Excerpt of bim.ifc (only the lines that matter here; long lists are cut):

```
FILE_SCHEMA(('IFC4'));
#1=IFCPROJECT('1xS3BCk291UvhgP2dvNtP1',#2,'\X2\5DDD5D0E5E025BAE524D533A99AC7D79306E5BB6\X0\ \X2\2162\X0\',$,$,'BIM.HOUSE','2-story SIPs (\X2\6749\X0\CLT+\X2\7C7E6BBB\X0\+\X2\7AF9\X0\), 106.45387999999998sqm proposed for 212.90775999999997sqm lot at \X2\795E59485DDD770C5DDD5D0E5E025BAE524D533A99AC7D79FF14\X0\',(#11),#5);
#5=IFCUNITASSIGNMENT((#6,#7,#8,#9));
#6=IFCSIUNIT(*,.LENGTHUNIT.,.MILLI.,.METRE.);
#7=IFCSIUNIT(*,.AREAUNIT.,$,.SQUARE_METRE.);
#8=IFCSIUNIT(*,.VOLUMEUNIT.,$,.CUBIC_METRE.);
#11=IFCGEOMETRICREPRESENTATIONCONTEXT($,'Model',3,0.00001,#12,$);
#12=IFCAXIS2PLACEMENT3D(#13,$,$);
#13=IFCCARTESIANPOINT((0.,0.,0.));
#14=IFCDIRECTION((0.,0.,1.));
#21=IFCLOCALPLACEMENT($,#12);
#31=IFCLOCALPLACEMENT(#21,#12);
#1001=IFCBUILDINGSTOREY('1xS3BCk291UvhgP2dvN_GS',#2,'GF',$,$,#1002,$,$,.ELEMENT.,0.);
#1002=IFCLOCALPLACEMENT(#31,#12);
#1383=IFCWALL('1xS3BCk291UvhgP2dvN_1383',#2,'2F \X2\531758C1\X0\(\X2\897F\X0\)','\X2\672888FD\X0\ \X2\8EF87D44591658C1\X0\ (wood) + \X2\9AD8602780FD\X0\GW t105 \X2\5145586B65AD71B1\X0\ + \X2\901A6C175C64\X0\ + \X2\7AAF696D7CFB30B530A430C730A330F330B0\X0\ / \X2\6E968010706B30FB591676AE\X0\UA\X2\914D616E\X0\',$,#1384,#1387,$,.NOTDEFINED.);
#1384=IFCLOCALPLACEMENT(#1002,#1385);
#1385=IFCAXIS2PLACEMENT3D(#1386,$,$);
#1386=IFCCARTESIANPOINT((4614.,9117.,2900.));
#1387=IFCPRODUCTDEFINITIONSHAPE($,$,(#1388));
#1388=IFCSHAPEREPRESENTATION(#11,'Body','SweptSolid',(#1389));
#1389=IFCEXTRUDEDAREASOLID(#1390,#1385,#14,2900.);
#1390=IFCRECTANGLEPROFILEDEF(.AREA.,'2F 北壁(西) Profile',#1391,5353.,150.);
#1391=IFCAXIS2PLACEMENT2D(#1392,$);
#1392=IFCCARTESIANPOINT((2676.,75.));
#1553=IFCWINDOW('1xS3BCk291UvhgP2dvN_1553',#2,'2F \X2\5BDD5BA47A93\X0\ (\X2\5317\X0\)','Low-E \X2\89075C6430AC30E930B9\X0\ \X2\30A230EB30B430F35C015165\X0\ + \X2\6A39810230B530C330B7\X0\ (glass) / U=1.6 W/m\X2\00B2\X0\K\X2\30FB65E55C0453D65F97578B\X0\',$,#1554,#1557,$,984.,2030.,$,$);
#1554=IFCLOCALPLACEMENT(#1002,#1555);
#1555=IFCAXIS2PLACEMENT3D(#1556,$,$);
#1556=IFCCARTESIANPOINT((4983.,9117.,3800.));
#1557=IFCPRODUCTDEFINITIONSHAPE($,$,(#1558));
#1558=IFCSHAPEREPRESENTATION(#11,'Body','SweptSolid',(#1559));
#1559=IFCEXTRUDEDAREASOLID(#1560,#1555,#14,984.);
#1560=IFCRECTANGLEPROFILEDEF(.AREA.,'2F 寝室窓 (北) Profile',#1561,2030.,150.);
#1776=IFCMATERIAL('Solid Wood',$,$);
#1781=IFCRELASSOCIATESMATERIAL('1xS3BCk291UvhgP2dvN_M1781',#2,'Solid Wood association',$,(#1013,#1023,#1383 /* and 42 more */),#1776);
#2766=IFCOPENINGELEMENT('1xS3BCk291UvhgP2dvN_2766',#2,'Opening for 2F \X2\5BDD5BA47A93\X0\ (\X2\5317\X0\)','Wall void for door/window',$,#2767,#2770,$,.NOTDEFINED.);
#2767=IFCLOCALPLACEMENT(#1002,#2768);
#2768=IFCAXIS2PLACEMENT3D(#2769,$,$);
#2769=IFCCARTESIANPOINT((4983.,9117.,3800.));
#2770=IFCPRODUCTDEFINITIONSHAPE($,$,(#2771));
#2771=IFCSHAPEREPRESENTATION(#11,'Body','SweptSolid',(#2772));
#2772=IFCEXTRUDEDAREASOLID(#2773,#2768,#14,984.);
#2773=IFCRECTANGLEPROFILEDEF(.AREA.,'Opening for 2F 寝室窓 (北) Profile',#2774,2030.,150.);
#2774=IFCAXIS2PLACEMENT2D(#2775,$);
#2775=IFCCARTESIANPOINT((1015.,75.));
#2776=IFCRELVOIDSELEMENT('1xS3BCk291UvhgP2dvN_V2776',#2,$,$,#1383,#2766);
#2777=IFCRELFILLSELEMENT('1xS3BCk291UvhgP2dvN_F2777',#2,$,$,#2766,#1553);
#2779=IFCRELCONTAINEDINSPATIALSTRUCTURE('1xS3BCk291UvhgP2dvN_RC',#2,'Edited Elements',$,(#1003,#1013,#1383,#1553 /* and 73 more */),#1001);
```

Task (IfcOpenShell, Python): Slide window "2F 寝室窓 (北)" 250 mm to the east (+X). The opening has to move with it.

```python
import ifcopenshell
import ifcopenshell.api.geometry
import ifcopenshell.util.placement

model = ifcopenshell.open("bim.ifc")

window = model.by_guid("1xS3BCk291UvhgP2dvN_1553")
opening = window.FillsVoids[0].RelatingOpeningElement
wall = opening.VoidsElements[0].RelatingBuildingElement

wall_matrix = ifcopenshell.util.placement.get_local_placement(wall.ObjectPlacement)
shift = wall_matrix[:3, 0] * 250.0
before = ifcopenshell.util.placement.get_local_placement(window.ObjectPlacement)[:3, 3].copy()

# The window is not placed relative to its opening, so move both.
for product in (opening, window):
    matrix = ifcopenshell.util.placement.get_local_placement(product.ObjectPlacement)
    matrix[:3, 3] += shift
    ifcopenshell.api.geometry.edit_object_placement(model, product=product, matrix=matrix, is_si=False)

after = ifcopenshell.util.placement.get_local_placement(window.ObjectPlacement)[:3, 3]
print("window moved by", (after - before).round(3) + 0.0)

model.write("bim_updated.ifc")
```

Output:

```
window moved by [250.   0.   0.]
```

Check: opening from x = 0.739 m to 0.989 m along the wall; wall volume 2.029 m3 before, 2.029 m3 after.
